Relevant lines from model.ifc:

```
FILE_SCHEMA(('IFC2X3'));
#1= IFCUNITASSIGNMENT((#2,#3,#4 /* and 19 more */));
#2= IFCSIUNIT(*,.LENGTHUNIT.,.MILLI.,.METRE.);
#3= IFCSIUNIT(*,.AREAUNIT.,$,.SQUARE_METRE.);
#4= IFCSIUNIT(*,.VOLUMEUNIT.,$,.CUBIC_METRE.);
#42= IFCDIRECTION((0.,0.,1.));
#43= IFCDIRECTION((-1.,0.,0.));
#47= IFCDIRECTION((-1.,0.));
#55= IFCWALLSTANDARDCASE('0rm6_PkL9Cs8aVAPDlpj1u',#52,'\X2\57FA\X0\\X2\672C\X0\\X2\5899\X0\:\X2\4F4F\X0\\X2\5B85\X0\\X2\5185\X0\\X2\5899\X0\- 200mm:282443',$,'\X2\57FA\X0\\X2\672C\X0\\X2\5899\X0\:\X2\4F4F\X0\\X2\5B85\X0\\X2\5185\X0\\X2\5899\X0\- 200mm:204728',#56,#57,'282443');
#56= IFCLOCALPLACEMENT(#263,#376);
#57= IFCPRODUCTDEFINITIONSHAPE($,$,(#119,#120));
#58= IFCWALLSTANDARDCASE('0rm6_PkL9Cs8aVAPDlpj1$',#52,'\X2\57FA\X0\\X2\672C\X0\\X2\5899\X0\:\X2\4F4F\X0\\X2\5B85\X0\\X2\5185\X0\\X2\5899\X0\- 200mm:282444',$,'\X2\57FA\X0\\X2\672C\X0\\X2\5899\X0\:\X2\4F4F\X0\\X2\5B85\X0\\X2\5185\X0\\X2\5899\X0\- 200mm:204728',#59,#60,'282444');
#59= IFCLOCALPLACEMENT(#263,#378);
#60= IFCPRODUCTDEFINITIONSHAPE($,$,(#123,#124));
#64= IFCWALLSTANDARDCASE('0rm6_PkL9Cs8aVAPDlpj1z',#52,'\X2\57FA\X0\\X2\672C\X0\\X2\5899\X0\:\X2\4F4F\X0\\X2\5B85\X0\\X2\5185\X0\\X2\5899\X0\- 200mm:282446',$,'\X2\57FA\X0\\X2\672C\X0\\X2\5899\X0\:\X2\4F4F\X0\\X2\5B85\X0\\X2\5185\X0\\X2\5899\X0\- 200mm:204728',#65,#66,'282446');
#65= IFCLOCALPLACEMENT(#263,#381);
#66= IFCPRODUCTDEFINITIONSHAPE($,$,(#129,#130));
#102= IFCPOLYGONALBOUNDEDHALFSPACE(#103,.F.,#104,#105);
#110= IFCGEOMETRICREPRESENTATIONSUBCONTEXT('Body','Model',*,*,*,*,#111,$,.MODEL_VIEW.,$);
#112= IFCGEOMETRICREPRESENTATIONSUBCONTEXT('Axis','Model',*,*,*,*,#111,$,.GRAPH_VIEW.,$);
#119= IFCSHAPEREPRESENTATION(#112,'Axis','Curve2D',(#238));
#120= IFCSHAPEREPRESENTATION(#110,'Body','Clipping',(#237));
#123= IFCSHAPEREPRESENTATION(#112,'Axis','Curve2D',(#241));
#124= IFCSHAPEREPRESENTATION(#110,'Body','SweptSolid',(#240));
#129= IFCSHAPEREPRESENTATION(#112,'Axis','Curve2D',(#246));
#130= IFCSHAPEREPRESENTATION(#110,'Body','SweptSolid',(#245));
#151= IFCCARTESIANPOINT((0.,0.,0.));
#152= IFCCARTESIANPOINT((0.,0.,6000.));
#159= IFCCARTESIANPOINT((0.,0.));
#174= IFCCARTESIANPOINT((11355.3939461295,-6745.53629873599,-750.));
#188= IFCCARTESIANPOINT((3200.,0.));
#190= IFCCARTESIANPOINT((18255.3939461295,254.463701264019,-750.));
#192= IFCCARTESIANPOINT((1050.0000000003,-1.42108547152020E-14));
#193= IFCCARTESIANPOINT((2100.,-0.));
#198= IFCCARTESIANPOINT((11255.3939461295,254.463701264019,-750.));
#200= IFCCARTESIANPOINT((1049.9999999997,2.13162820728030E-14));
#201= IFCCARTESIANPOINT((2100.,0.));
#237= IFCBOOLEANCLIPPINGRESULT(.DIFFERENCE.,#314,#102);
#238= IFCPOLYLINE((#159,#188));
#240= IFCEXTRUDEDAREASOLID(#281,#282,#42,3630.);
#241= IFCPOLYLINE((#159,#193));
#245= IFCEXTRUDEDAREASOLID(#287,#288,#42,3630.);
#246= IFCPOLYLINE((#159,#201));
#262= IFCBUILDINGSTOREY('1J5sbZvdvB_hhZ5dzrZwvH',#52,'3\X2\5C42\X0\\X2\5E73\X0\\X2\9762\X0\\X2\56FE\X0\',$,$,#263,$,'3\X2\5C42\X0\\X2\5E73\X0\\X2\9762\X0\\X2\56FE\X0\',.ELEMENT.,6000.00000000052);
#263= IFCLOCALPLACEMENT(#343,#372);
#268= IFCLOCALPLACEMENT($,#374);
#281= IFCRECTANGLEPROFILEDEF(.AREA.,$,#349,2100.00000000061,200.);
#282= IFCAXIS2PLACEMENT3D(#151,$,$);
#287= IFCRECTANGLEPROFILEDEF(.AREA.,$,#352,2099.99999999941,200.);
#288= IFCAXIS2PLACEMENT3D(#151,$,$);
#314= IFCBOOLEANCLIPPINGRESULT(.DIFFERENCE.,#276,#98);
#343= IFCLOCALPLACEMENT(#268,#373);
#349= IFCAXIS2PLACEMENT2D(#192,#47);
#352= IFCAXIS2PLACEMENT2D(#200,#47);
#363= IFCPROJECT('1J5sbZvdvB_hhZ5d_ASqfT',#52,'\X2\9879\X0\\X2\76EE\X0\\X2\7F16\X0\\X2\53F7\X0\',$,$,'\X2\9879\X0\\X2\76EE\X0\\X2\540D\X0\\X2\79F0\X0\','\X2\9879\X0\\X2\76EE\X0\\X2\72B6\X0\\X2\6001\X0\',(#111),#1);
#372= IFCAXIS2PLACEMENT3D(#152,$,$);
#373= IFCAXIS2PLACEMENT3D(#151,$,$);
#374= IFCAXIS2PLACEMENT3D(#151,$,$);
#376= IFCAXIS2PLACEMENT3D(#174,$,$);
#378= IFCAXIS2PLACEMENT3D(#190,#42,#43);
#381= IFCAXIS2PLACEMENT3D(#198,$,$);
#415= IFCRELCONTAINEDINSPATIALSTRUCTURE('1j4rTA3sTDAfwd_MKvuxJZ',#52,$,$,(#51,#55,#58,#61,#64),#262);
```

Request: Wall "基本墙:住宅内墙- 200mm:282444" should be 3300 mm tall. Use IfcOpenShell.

```python
import ifcopenshell
import ifcopenshell.geom
import ifcopenshell.util.representation
import ifcopenshell.util.shape
import ifcopenshell.util.unit

model = ifcopenshell.open("model.ifc")
unit_scale = ifcopenshell.util.unit.calculate_unit_scale(model)
settings = ifcopenshell.geom.settings()


def volume(element):
    """Net volume in cubic metres, openings subtracted."""
    shape = ifcopenshell.geom.create_shape(settings, element)
    return ifcopenshell.util.shape.get_volume(shape.geometry)


wall = model.by_guid("0rm6_PkL9Cs8aVAPDlpj1$")
before = volume(wall)

body = ifcopenshell.util.representation.get_representation(wall, "Model", "Body")
solid = body.Items[0]
old_height = solid.Depth
solid.Depth = 3.3 / unit_scale
after = volume(wall)

print(f"height {old_height:g} -> {solid.Depth:g}, volume {before:.3f} -> {after:.3f} m3")

model.write("model_v2.ifc")
```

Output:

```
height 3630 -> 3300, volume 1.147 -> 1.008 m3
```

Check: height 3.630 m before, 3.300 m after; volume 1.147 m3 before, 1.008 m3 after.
